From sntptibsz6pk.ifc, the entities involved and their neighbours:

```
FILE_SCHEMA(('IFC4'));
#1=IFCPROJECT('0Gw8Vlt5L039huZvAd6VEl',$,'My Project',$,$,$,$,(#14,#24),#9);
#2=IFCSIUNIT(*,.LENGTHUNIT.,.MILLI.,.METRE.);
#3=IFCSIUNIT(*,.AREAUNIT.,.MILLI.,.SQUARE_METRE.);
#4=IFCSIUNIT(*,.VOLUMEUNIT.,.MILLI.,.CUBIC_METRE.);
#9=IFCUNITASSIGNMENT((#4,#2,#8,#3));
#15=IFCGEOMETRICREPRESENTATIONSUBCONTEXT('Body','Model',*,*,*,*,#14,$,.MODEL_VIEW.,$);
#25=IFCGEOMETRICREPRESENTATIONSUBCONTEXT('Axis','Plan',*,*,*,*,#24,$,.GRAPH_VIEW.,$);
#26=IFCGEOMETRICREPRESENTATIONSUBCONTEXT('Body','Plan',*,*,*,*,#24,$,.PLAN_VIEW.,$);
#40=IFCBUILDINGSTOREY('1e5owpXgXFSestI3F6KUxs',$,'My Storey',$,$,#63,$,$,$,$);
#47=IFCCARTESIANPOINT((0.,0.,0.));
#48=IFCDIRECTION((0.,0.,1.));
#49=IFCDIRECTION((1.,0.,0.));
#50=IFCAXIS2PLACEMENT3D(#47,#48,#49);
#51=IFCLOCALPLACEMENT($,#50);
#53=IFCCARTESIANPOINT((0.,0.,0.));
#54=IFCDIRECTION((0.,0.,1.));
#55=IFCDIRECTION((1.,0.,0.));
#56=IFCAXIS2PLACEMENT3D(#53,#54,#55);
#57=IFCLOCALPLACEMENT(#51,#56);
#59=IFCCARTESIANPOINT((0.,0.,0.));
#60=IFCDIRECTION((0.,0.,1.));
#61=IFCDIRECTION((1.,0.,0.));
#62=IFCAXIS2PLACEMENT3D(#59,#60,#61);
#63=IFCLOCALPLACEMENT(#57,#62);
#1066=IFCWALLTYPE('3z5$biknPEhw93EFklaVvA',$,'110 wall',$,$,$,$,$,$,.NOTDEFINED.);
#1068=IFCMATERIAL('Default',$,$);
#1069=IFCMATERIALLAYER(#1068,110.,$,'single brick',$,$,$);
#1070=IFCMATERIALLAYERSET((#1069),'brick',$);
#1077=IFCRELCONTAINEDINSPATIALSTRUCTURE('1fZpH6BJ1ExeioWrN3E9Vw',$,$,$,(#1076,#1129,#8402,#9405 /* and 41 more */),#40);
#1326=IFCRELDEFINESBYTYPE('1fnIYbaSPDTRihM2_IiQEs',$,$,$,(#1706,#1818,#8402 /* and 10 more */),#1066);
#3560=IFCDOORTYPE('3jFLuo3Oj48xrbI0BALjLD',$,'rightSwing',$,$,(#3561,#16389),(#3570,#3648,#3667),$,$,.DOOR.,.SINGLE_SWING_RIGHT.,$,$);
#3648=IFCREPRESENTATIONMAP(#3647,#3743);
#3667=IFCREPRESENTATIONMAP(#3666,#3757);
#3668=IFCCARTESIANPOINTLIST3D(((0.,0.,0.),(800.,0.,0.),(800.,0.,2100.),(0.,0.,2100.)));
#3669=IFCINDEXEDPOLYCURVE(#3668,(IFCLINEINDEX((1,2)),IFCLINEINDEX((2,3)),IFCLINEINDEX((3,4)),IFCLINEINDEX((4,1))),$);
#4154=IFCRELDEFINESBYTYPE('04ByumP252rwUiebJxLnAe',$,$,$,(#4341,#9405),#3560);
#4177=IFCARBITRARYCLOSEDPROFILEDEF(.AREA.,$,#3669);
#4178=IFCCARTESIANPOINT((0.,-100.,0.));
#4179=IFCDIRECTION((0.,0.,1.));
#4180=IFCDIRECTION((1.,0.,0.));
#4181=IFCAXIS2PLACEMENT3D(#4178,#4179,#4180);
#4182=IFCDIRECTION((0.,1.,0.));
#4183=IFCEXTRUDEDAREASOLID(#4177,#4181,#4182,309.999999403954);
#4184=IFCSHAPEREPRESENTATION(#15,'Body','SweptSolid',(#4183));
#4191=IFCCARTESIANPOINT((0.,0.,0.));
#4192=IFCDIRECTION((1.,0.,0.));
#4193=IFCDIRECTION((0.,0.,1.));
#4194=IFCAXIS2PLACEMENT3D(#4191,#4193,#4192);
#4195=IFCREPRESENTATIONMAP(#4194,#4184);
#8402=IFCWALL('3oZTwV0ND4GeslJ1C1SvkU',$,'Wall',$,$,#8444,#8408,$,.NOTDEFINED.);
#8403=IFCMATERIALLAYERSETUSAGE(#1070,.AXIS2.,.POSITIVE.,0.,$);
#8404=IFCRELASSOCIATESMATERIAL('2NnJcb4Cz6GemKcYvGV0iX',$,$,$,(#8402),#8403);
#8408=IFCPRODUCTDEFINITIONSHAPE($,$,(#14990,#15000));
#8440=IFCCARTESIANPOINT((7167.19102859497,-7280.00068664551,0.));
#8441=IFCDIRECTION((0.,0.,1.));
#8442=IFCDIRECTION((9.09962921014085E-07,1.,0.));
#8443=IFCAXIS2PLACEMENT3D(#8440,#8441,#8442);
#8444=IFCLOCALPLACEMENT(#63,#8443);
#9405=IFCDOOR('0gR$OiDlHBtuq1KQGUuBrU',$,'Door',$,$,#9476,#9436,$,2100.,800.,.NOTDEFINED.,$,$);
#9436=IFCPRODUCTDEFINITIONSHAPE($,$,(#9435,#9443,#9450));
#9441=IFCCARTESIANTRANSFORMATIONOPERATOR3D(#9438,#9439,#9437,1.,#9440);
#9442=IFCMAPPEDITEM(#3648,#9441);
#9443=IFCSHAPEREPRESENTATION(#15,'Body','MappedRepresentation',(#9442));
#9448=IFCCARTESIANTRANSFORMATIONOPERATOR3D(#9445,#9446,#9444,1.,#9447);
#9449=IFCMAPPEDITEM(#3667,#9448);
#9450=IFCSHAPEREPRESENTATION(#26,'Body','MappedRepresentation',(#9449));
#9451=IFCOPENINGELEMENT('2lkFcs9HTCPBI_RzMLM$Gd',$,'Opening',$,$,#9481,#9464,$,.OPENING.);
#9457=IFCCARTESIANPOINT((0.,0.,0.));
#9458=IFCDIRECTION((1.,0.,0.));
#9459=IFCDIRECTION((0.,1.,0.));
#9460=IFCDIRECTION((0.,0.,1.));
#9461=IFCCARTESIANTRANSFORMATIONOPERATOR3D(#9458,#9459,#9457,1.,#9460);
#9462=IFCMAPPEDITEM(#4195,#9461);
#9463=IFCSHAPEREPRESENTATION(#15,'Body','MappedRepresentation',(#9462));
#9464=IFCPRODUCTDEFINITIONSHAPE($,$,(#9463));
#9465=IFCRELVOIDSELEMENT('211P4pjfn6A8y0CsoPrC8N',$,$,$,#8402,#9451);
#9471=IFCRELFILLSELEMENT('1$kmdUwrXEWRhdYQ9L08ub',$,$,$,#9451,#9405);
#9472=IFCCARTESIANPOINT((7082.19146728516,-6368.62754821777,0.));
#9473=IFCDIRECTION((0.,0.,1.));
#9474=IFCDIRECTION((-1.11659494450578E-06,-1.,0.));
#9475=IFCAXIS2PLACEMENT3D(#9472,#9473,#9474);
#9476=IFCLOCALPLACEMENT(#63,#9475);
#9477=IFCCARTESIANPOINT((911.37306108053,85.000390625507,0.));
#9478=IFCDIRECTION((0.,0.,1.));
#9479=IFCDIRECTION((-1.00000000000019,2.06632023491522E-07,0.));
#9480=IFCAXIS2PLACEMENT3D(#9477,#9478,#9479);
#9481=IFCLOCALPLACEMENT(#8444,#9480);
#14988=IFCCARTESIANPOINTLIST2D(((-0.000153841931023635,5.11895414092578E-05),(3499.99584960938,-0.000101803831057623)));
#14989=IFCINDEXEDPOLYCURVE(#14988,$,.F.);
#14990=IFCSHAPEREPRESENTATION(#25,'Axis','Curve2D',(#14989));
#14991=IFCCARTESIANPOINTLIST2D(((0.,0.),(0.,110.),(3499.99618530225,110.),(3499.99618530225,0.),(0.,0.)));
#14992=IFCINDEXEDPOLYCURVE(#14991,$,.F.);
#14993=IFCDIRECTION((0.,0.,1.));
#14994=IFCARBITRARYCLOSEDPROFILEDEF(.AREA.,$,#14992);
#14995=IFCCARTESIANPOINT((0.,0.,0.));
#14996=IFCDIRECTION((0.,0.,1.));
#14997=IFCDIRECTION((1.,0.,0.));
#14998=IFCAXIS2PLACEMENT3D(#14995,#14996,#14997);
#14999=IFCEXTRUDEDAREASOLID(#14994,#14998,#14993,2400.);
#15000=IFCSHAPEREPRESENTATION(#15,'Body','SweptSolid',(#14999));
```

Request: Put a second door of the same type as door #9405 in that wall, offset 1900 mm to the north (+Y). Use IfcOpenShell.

```python
import ifcopenshell
import ifcopenshell.api.feature
import ifcopenshell.api.geometry
import ifcopenshell.api.root
import ifcopenshell.geom
import ifcopenshell.util.element
import ifcopenshell.util.placement
import ifcopenshell.util.shape

model = ifcopenshell.open("sntptibsz6pk.ifc")
settings = ifcopenshell.geom.settings()


def volume(element):
    """Net volume in cubic metres, openings subtracted."""
    shape = ifcopenshell.geom.create_shape(settings, element)
    return ifcopenshell.util.shape.get_volume(shape.geometry)


door = model.by_id(9405)
opening = door.FillsVoids[0].RelatingOpeningElement
wall = opening.VoidsElements[0].RelatingBuildingElement
before = volume(wall)
shift = ifcopenshell.util.placement.get_local_placement(wall.ObjectPlacement)[:3, 0] * 1900.0

# copy_class copies the void relationship, type, container and properties, but no geometry.
new_opening = ifcopenshell.api.root.copy_class(model, product=opening)
new_opening.Representation = ifcopenshell.util.element.copy_deep(
    model, opening.Representation, exclude=["IfcGeometricRepresentationContext", "IfcRepresentationMap"]
)
new_door = ifcopenshell.api.root.copy_class(model, product=door)
new_door.Representation = ifcopenshell.util.element.copy_deep(
    model, door.Representation, exclude=["IfcGeometricRepresentationContext", "IfcRepresentationMap"]
)
ifcopenshell.api.feature.add_filling(model, opening=new_opening, element=new_door)

for old, new in ((opening, new_opening), (door, new_door)):
    matrix = ifcopenshell.util.placement.get_local_placement(old.ObjectPlacement)
    matrix[:3, 3] += shift
    ifcopenshell.api.geometry.edit_object_placement(model, product=new, matrix=matrix, is_si=False)

after = volume(wall)

print(f"wall volume {before:.3f} -> {after:.3f} m3")

model.write("sntptibsz6pk_v2.ifc")
```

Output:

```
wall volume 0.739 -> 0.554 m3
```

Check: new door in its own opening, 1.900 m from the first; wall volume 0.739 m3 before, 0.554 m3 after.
